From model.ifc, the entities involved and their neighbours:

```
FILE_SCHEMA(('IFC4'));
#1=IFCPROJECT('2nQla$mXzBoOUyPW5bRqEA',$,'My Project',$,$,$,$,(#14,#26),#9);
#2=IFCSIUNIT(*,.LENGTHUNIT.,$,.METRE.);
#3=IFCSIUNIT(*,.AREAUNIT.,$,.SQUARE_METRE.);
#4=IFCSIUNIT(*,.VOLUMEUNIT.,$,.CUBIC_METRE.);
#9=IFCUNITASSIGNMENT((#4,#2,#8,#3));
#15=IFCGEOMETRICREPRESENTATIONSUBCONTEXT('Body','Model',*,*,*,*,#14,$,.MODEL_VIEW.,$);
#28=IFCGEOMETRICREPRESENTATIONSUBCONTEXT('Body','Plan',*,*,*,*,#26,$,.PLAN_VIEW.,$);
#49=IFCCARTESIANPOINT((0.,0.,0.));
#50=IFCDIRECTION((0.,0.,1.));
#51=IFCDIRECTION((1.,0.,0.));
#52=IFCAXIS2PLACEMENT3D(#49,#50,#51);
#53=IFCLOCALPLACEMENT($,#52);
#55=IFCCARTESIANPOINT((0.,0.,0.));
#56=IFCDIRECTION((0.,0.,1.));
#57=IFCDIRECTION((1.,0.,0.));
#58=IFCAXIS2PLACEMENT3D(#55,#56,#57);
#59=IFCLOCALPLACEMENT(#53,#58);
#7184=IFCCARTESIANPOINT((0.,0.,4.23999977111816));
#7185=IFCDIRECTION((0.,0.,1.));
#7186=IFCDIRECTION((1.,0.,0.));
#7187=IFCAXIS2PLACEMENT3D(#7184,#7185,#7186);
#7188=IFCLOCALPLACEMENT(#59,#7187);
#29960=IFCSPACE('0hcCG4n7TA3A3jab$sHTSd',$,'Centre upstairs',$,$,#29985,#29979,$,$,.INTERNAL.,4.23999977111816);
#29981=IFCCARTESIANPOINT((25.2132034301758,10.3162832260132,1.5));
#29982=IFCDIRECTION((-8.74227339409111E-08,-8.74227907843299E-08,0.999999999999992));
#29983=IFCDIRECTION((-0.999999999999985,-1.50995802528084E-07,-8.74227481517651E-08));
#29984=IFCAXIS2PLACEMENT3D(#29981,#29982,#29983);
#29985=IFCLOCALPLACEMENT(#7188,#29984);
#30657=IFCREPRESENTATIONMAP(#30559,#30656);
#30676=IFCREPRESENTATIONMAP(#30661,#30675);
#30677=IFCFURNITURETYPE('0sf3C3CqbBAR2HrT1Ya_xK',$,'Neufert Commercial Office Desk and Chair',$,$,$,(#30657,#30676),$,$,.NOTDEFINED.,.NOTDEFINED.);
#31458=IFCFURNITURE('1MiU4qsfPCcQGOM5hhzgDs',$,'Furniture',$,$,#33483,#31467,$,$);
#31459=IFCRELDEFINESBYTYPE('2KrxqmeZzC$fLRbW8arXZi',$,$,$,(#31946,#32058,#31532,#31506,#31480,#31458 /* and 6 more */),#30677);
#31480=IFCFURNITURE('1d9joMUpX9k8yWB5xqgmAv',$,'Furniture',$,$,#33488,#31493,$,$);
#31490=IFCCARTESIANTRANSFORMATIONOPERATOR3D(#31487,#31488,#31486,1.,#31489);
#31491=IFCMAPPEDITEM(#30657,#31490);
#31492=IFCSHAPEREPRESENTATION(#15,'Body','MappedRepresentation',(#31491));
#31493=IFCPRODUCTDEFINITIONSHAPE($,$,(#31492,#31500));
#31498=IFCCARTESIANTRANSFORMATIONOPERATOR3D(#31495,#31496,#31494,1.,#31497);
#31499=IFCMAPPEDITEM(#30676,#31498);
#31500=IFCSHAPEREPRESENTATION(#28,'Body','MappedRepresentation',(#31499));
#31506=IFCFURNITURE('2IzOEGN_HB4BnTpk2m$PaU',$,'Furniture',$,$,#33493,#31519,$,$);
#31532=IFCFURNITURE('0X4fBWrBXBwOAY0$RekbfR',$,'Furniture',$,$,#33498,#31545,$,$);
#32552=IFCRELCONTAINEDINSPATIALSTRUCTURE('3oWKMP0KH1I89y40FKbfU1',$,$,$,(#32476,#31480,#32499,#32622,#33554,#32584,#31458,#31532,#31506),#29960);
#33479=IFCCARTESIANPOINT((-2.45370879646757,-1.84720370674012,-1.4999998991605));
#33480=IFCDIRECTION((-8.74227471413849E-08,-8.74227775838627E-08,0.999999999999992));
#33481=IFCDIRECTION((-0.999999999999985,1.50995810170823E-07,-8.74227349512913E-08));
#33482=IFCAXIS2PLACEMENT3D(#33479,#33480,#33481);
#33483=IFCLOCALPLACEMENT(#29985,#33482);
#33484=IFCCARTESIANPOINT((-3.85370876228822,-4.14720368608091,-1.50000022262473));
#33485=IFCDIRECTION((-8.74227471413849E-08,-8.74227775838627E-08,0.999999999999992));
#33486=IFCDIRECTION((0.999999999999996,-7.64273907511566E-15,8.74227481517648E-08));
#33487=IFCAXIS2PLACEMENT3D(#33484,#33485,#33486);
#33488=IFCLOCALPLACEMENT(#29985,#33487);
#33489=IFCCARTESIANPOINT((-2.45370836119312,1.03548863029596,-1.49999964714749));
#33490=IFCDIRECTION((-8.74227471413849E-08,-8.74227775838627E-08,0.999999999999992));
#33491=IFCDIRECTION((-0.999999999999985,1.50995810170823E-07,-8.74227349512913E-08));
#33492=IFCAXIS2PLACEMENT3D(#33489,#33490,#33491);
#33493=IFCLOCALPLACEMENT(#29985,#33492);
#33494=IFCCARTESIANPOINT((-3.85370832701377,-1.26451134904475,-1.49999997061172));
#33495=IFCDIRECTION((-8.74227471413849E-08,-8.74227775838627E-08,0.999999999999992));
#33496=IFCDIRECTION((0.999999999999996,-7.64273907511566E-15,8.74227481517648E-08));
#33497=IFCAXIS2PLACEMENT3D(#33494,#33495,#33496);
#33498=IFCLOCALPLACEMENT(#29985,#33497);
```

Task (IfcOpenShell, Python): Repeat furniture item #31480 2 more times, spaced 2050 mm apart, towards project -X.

```python
import numpy as np
import ifcopenshell
import ifcopenshell.api.geometry
import ifcopenshell.api.root
import ifcopenshell.util.element
import ifcopenshell.util.placement
import ifcopenshell.util.unit

model = ifcopenshell.open("model.ifc")
unit_scale = ifcopenshell.util.unit.calculate_unit_scale(model)

source = model.by_guid("1d9joMUpX9k8yWB5xqgmAv")
base = ifcopenshell.util.placement.get_local_placement(source.ObjectPlacement)
step = np.array([-1.0, 0.0, 0.0]) * 2.05 / unit_scale

for i in range(1, 3):
    copy = ifcopenshell.api.root.copy_class(model, product=source)
    copy.Representation = ifcopenshell.util.element.copy_deep(
        model, source.Representation, exclude=["IfcGeometricRepresentationContext", "IfcRepresentationMap"]
    )
    matrix = base.copy()
    matrix[:3, 3] += i * step
    print("added at", matrix[:3, 3].round(3) + 0.0)
    ifcopenshell.api.geometry.edit_object_placement(model, product=copy, matrix=matrix, is_si=False)

model.write("model-out.ifc")
```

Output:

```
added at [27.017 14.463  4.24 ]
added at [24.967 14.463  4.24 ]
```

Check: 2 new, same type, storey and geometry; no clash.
